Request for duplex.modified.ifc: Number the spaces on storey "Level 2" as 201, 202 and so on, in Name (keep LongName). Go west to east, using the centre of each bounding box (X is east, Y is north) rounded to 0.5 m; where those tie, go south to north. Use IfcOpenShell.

First a look at what the model holds.

```python
import ifcopenshell
import ifcopenshell.util.element
import ifcopenshell.util.placement

model = ifcopenshell.open("duplex.modified.ifc")
print(model.schema)
storey = next(s for s in model.by_type("IfcBuildingStorey") if s.Name == "Level 2")
spaces = [e for e in ifcopenshell.util.element.get_decomposition(storey) if e.is_a("IfcSpace")]
for e in sorted(spaces, key=lambda e: e.id()):
    origin = ifcopenshell.util.placement.get_local_placement(e.ObjectPlacement)[:3, 3]
    print(e.id(), e.Name, e.LongName, origin.round(2) + 0.0, sep=" | ")
```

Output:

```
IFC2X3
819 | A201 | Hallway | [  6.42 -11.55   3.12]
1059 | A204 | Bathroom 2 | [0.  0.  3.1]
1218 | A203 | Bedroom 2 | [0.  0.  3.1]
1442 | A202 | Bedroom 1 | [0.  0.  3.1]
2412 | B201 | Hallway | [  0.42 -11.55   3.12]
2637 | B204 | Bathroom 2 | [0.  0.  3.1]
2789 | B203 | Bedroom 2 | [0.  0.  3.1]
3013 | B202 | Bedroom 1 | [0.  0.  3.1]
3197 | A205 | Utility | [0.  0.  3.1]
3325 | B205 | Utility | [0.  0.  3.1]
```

```python
import ifcopenshell
import ifcopenshell.geom
import ifcopenshell.util.element
import ifcopenshell.util.shape

model = ifcopenshell.open("duplex.modified.ifc")
settings = ifcopenshell.geom.settings()
settings.set("use-world-coords", True)


def centre(element):
    shape = ifcopenshell.geom.create_shape(settings, element)
    return ifcopenshell.util.shape.get_bbox_centroid(shape.geometry)


storey = next(s for s in model.by_type("IfcBuildingStorey") if s.Name == "Level 2")
spaces = [e for e in ifcopenshell.util.element.get_decomposition(storey) if e.is_a("IfcSpace")]

# Insertion points can sit at a corner or the storey origin, so sort by the geometry (in metres).
centres = {e: centre(e) for e in spaces}
spaces.sort(key=lambda e: (round(centres[e][0] / 0.5), centres[e][1]))

for i, e in enumerate(spaces, start=1):
    number = f"2{i:02d}"
    e.Name = number
    print(e.id(), number)

model.write("duplex.modified_v2.ifc")
```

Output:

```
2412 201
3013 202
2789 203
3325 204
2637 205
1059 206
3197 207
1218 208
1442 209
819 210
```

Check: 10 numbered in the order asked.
